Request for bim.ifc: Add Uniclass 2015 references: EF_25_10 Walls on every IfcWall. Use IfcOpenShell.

First a look at what the model holds.

```python
import ifcopenshell

model = ifcopenshell.open("bim.ifc")
print(model.schema)
print("classifications:", [c.Name for c in model.by_type("IfcClassification")])
for ifc_class in ("IfcDoor", "IfcRoof", "IfcStair", "IfcWall", "IfcWindow"):
    print(ifc_class, len(model.by_type(ifc_class)))
```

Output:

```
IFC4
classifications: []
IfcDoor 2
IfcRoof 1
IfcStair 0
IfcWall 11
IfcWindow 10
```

```python
import ifcopenshell
import ifcopenshell.api.classification

model = ifcopenshell.open("bim.ifc")

system = ifcopenshell.api.classification.add_classification(model, classification="Uniclass 2015")

codes = {
    "IfcWall": ("EF_25_10", "Walls"),
}
for ifc_class, (code, name) in codes.items():
    products = model.by_type(ifc_class)
    ifcopenshell.api.classification.add_reference(
        model, products=products, classification=system, identification=code, name=name
    )
    print(code, len(products))

model.write("bim_edited.ifc")
```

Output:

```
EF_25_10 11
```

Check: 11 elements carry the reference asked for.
